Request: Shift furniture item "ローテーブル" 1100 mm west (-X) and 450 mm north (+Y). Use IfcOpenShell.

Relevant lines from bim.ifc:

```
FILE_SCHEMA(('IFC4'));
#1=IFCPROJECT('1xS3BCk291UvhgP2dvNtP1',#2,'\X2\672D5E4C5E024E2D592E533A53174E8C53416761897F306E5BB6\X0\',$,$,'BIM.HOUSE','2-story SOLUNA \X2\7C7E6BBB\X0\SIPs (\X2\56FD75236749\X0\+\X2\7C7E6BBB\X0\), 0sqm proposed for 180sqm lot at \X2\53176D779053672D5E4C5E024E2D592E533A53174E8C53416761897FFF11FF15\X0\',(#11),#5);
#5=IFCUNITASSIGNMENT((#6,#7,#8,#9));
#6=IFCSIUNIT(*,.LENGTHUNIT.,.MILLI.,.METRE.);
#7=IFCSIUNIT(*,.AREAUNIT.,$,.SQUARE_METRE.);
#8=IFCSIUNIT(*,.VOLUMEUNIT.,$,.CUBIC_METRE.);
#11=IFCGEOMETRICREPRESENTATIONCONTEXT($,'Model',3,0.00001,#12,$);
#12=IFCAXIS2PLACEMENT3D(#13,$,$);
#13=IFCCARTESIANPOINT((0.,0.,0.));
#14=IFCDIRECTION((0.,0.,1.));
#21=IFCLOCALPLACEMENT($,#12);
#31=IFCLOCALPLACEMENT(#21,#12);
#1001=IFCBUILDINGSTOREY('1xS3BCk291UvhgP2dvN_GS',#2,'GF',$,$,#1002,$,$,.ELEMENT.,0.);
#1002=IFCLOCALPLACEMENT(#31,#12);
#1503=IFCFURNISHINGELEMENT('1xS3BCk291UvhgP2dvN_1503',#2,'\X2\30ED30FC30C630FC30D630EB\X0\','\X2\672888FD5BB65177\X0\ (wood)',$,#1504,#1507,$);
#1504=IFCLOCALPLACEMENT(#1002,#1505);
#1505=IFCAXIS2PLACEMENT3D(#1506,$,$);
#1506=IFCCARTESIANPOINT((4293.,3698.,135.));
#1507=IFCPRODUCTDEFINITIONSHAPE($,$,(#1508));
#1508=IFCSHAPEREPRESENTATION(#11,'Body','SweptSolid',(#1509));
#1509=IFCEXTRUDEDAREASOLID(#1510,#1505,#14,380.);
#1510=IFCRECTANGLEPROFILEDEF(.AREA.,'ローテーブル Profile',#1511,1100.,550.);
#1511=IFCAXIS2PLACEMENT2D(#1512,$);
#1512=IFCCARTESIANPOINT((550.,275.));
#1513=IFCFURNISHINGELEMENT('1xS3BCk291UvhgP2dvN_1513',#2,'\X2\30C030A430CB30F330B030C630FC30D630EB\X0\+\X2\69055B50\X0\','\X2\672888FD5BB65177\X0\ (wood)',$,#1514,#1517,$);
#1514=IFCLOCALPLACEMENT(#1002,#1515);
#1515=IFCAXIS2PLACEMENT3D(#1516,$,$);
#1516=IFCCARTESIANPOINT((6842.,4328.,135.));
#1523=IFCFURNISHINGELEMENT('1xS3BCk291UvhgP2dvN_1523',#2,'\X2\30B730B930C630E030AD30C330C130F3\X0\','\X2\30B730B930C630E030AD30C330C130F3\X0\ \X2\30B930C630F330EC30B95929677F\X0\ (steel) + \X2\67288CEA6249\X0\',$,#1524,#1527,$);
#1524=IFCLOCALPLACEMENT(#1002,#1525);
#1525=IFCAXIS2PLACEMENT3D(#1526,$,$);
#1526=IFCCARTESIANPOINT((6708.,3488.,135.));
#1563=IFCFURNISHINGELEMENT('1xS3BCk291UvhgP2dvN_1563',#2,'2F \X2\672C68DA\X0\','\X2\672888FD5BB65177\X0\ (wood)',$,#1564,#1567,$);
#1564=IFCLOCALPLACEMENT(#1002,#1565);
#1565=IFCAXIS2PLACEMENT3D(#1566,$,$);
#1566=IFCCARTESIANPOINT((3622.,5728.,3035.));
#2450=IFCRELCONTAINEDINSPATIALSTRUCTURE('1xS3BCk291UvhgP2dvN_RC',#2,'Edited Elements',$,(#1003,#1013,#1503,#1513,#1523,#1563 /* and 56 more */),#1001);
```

```python
import ifcopenshell
import ifcopenshell.api.geometry
import ifcopenshell.util.placement
import ifcopenshell.util.unit

model = ifcopenshell.open("bim.ifc")
unit_scale = ifcopenshell.util.unit.calculate_unit_scale(model)

item = model.by_guid("1xS3BCk291UvhgP2dvN_1503")
matrix = ifcopenshell.util.placement.get_local_placement(item.ObjectPlacement)
matrix[0, 3] -= 1.1 / unit_scale
matrix[1, 3] += 0.45 / unit_scale
ifcopenshell.api.geometry.edit_object_placement(model, product=item, matrix=matrix, is_si=False)

print(ifcopenshell.util.placement.get_local_placement(item.ObjectPlacement).round(3) + 0.0)

model.write("bim_updated.ifc")
```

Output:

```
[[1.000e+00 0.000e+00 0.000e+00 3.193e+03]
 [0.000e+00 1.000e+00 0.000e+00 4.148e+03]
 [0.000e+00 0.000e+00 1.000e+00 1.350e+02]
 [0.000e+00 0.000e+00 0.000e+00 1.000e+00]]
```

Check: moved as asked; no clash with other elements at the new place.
